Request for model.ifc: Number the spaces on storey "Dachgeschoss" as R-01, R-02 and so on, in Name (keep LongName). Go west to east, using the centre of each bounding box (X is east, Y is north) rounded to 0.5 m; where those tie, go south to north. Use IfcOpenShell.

First a look at what the model holds.

```python
import ifcopenshell
import ifcopenshell.util.element
import ifcopenshell.util.placement

model = ifcopenshell.open("model.ifc")
print(model.schema)
storey = next(s for s in model.by_type("IfcBuildingStorey") if s.Name == "Dachgeschoss")
spaces = [e for e in ifcopenshell.util.element.get_decomposition(storey) if e.is_a("IfcSpace")]
for e in sorted(spaces, key=lambda e: e.id()):
    origin = ifcopenshell.util.placement.get_local_placement(e.ObjectPlacement)[:3, 3]
    print(e.id(), e.Name, e.LongName, origin.round(2) + 0.0, sep=" | ")
```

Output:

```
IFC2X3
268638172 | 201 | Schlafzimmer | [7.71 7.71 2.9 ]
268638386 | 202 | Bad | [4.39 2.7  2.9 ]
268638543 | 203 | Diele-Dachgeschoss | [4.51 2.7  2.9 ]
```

```python
import ifcopenshell
import ifcopenshell.geom
import ifcopenshell.util.element
import ifcopenshell.util.shape

model = ifcopenshell.open("model.ifc")
settings = ifcopenshell.geom.settings()
settings.set("use-world-coords", True)


def centre(element):
    shape = ifcopenshell.geom.create_shape(settings, element)
    return ifcopenshell.util.shape.get_bbox_centroid(shape.geometry)


storey = next(s for s in model.by_type("IfcBuildingStorey") if s.Name == "Dachgeschoss")
spaces = [e for e in ifcopenshell.util.element.get_decomposition(storey) if e.is_a("IfcSpace")]

# Insertion points can sit at a corner or the storey origin, so sort by the geometry (in metres).
centres = {e: centre(e) for e in spaces}
spaces.sort(key=lambda e: (round(centres[e][0] / 0.5), centres[e][1]))

for i, e in enumerate(spaces, start=1):
    number = f"R-{i:02d}"
    e.Name = number
    print(e.id(), number)

model.write("model_v2.ifc")
```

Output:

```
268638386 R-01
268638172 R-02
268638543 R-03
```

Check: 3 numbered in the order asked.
